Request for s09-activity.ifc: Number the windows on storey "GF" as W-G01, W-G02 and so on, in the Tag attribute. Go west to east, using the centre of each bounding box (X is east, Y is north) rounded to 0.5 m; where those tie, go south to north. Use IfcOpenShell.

First a look at what the model holds.

```python
import ifcopenshell
import ifcopenshell.util.element
import ifcopenshell.util.placement

model = ifcopenshell.open("s09-activity.ifc")
print(model.schema)
storey = next(s for s in model.by_type("IfcBuildingStorey") if s.Name == "GF")
windows = [e for e in ifcopenshell.util.element.get_decomposition(storey) if e.is_a("IfcWindow")]
for e in sorted(windows, key=lambda e: e.id()):
    origin = ifcopenshell.util.placement.get_local_placement(e.ObjectPlacement)[:3, 3]
    print(e.id(), e.Tag, e.Name, origin.round(2) + 0.0, sep=" | ")
```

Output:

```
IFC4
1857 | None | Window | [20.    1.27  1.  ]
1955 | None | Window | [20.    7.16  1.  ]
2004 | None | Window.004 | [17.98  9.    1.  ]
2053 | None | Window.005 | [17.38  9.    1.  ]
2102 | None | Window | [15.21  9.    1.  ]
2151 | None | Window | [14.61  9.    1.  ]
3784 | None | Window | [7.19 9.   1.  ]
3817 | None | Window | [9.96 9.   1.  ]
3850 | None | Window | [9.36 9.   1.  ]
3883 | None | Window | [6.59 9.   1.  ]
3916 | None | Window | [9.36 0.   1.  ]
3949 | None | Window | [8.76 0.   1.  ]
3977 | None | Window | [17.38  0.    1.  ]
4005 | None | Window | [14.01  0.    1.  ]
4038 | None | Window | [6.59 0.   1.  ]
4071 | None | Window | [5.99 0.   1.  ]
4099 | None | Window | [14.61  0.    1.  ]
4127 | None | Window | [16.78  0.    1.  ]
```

```python
import ifcopenshell
import ifcopenshell.geom
import ifcopenshell.util.element
import ifcopenshell.util.shape

model = ifcopenshell.open("s09-activity.ifc")
settings = ifcopenshell.geom.settings()
settings.set("use-world-coords", True)


def centre(element):
    shape = ifcopenshell.geom.create_shape(settings, element)
    return ifcopenshell.util.shape.get_bbox_centroid(shape.geometry)


storey = next(s for s in model.by_type("IfcBuildingStorey") if s.Name == "GF")
windows = [e for e in ifcopenshell.util.element.get_decomposition(storey) if e.is_a("IfcWindow")]

# Insertion points can sit at a corner or the storey origin, so sort by the geometry (in metres).
centres = {e: centre(e) for e in windows}
windows.sort(key=lambda e: (round(centres[e][0] / 0.5), centres[e][1]))

for i, e in enumerate(windows, start=1):
    number = f"W-G{i:02d}"
    e.Tag = number
    print(e.id(), number)

model.write("s09-activity-out.ifc")
```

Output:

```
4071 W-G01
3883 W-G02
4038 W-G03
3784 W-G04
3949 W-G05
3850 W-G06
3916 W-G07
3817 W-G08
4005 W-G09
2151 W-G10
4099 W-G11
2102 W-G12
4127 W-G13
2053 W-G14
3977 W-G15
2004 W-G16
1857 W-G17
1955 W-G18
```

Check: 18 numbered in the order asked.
